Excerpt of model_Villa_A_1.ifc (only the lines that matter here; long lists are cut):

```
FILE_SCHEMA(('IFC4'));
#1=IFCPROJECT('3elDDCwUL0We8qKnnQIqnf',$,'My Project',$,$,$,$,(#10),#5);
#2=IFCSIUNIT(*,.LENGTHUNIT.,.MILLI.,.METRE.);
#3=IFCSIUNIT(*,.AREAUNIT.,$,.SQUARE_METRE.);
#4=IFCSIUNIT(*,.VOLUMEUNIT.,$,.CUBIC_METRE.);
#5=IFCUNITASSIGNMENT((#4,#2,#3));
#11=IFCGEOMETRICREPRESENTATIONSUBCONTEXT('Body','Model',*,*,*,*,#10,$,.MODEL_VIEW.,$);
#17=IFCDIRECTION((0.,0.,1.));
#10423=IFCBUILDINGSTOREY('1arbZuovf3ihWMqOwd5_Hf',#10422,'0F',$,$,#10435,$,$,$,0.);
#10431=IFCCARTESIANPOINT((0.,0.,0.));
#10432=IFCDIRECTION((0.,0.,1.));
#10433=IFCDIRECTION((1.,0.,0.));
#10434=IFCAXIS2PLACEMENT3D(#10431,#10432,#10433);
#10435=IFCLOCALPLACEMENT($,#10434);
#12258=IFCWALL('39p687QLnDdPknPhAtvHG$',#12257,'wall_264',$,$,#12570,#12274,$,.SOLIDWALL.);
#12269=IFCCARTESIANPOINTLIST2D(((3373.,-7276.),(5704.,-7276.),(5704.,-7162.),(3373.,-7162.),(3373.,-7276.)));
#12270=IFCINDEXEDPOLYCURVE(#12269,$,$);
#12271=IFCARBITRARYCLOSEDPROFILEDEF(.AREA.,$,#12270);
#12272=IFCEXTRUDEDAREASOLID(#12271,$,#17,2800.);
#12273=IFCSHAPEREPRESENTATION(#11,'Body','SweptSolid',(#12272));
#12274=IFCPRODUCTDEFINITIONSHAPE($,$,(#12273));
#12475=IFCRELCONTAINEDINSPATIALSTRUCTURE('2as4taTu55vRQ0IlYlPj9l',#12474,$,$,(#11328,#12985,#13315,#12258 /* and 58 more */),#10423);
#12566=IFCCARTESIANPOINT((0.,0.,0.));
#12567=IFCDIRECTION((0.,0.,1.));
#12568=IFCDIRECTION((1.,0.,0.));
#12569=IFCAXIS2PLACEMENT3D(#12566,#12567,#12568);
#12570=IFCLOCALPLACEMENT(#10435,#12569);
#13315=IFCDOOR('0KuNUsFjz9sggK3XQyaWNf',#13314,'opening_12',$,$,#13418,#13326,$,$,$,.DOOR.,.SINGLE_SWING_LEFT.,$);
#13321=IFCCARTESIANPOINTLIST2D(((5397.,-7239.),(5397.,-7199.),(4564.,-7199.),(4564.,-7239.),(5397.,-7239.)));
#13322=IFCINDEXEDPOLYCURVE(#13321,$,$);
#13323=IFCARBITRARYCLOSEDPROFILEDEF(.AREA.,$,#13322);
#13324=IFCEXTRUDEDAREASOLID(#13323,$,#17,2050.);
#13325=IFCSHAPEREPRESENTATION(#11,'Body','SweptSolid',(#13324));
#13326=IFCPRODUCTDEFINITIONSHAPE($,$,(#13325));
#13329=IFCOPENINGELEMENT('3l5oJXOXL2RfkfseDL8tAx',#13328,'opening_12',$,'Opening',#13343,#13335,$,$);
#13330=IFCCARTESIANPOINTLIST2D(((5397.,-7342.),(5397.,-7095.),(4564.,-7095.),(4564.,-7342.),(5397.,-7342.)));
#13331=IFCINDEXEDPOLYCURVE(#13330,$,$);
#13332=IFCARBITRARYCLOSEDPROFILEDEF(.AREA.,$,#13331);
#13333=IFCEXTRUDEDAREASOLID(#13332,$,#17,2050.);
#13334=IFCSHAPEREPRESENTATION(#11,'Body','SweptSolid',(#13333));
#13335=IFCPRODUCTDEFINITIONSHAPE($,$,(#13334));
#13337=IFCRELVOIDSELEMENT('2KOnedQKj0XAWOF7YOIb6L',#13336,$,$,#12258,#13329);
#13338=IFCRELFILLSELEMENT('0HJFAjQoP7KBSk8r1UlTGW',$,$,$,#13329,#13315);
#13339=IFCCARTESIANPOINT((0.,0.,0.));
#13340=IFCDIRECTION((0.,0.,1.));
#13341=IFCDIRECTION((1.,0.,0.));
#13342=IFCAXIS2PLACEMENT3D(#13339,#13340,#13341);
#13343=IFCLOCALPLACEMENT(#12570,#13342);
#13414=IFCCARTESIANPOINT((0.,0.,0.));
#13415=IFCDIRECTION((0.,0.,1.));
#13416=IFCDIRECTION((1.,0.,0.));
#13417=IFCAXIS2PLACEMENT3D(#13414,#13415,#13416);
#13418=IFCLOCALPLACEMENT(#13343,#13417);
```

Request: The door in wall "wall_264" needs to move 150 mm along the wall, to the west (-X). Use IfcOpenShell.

```python
import ifcopenshell
import ifcopenshell.api.geometry
import ifcopenshell.util.placement

model = ifcopenshell.open("model_Villa_A_1.ifc")

door = model.by_guid("0KuNUsFjz9sggK3XQyaWNf")
opening = door.FillsVoids[0].RelatingOpeningElement
wall = opening.VoidsElements[0].RelatingBuildingElement

wall_matrix = ifcopenshell.util.placement.get_local_placement(wall.ObjectPlacement)
shift = wall_matrix[:3, 0] * -150.0
before = ifcopenshell.util.placement.get_local_placement(door.ObjectPlacement)[:3, 3].copy()

# The door is placed relative to its opening, so it follows when the opening moves.
matrix = ifcopenshell.util.placement.get_local_placement(opening.ObjectPlacement)
matrix[:3, 3] += shift
ifcopenshell.api.geometry.edit_object_placement(
    model, product=opening, matrix=matrix, is_si=False, should_transform_children=True
)

after = ifcopenshell.util.placement.get_local_placement(door.ObjectPlacement)[:3, 3]
print("door moved by", (after - before).round(3) + 0.0)

model.write("model_Villa_A_1_rev.ifc")
```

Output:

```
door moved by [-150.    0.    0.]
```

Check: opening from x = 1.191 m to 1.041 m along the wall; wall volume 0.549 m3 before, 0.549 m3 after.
